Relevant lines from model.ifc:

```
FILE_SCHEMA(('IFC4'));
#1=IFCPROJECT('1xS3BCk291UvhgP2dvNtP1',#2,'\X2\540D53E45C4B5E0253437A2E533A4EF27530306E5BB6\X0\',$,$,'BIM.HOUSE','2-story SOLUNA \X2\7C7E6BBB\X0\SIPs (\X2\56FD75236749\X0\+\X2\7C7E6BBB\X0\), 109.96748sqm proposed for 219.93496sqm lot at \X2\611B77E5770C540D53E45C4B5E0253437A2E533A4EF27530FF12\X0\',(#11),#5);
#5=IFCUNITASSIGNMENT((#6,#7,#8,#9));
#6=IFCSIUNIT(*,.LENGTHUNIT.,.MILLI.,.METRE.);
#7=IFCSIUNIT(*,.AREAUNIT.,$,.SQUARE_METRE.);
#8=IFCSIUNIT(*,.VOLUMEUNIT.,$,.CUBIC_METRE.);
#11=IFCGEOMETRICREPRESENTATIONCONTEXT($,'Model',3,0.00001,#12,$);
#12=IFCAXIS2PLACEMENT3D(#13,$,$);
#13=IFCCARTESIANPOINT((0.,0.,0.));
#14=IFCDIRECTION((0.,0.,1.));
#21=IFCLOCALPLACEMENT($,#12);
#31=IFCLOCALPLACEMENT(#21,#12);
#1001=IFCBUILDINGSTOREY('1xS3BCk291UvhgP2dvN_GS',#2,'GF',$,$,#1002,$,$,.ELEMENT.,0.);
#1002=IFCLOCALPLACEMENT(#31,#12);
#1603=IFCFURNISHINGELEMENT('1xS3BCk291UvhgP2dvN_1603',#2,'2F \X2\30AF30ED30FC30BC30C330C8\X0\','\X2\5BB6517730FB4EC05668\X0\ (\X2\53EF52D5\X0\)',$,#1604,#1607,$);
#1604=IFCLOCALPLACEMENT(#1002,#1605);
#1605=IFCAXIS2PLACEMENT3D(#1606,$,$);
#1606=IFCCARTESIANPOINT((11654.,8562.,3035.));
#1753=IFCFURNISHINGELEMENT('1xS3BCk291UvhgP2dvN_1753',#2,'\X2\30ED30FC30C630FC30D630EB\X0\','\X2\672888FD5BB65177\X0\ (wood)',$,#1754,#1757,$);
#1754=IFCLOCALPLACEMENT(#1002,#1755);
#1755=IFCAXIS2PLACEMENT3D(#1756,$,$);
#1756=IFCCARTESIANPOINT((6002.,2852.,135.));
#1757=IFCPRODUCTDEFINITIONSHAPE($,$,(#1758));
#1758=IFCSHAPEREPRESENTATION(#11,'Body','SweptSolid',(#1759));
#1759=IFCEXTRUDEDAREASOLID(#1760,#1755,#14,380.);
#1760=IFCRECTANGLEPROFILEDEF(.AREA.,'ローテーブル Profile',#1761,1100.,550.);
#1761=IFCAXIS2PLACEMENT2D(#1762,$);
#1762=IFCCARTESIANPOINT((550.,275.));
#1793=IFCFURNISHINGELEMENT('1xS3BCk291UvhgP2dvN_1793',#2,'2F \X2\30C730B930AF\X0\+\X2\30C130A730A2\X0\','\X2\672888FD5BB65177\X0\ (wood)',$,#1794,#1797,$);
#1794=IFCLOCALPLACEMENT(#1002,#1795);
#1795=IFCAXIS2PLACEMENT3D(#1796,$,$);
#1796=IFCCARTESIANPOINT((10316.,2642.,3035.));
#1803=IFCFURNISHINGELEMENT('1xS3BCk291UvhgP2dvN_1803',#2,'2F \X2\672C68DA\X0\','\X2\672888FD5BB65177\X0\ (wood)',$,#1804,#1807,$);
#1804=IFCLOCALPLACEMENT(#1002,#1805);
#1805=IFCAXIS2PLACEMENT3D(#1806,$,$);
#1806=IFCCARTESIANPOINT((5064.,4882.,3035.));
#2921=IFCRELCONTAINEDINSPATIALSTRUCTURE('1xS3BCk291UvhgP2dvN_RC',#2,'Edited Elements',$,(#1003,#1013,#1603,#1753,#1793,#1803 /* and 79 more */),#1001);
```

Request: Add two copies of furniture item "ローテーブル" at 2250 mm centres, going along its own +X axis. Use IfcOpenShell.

```python
import ifcopenshell
import ifcopenshell.api.geometry
import ifcopenshell.api.root
import ifcopenshell.util.element
import ifcopenshell.util.placement

model = ifcopenshell.open("model.ifc")


def reuse_history(source, copy):
    """copy_class also copies each property set's owner history, people and application; keep the originals."""
    for rel in copy.IsDefinedBy:
        if rel.is_a("IfcRelDefinesByProperties") and (history := rel.RelatingPropertyDefinition.OwnerHistory):
            rel.RelatingPropertyDefinition.OwnerHistory = source.OwnerHistory
            ifcopenshell.util.element.remove_deep2(model, history)


source = model.by_guid("1xS3BCk291UvhgP2dvN_1753")
base = ifcopenshell.util.placement.get_local_placement(source.ObjectPlacement)
step = base[:3, 0] * 2250.0

for i in range(1, 3):
    copy = ifcopenshell.api.root.copy_class(model, product=source)
    copy.Representation = ifcopenshell.util.element.copy_deep(
        model, source.Representation, exclude=["IfcGeometricRepresentationContext", "IfcRepresentationMap"]
    )
    reuse_history(source, copy)
    matrix = base.copy()
    matrix[:3, 3] += i * step
    print("added at", matrix[:3, 3].round(3) + 0.0)
    ifcopenshell.api.geometry.edit_object_placement(model, product=copy, matrix=matrix, is_si=False)

model.write("model_edited.ifc")
```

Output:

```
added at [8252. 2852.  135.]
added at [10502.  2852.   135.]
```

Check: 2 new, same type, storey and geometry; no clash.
